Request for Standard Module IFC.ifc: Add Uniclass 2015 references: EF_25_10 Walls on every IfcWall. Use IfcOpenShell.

First a look at what the model holds.

```python
import ifcopenshell

model = ifcopenshell.open("Standard Module IFC.ifc")
print(model.schema)
print("classifications:", [c.Name for c in model.by_type("IfcClassification")])
for ifc_class in ("IfcDoor", "IfcRoof", "IfcStair", "IfcWall", "IfcWindow"):
    print(ifc_class, len(model.by_type(ifc_class)))
```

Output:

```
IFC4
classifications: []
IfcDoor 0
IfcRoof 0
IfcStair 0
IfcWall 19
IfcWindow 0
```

```python
import ifcopenshell
import ifcopenshell.api.classification

model = ifcopenshell.open("Standard Module IFC.ifc")

system = ifcopenshell.api.classification.add_classification(model, classification="Uniclass 2015")

codes = {
    "IfcWall": ("EF_25_10", "Walls"),
}
for ifc_class, (code, name) in codes.items():
    products = model.by_type(ifc_class)
    ifcopenshell.api.classification.add_reference(
        model, products=products, classification=system, identification=code, name=name
    )
    print(code, len(products))

model.write("Standard Module IFC_rev.ifc")
```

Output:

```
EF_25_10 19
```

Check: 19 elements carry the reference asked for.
